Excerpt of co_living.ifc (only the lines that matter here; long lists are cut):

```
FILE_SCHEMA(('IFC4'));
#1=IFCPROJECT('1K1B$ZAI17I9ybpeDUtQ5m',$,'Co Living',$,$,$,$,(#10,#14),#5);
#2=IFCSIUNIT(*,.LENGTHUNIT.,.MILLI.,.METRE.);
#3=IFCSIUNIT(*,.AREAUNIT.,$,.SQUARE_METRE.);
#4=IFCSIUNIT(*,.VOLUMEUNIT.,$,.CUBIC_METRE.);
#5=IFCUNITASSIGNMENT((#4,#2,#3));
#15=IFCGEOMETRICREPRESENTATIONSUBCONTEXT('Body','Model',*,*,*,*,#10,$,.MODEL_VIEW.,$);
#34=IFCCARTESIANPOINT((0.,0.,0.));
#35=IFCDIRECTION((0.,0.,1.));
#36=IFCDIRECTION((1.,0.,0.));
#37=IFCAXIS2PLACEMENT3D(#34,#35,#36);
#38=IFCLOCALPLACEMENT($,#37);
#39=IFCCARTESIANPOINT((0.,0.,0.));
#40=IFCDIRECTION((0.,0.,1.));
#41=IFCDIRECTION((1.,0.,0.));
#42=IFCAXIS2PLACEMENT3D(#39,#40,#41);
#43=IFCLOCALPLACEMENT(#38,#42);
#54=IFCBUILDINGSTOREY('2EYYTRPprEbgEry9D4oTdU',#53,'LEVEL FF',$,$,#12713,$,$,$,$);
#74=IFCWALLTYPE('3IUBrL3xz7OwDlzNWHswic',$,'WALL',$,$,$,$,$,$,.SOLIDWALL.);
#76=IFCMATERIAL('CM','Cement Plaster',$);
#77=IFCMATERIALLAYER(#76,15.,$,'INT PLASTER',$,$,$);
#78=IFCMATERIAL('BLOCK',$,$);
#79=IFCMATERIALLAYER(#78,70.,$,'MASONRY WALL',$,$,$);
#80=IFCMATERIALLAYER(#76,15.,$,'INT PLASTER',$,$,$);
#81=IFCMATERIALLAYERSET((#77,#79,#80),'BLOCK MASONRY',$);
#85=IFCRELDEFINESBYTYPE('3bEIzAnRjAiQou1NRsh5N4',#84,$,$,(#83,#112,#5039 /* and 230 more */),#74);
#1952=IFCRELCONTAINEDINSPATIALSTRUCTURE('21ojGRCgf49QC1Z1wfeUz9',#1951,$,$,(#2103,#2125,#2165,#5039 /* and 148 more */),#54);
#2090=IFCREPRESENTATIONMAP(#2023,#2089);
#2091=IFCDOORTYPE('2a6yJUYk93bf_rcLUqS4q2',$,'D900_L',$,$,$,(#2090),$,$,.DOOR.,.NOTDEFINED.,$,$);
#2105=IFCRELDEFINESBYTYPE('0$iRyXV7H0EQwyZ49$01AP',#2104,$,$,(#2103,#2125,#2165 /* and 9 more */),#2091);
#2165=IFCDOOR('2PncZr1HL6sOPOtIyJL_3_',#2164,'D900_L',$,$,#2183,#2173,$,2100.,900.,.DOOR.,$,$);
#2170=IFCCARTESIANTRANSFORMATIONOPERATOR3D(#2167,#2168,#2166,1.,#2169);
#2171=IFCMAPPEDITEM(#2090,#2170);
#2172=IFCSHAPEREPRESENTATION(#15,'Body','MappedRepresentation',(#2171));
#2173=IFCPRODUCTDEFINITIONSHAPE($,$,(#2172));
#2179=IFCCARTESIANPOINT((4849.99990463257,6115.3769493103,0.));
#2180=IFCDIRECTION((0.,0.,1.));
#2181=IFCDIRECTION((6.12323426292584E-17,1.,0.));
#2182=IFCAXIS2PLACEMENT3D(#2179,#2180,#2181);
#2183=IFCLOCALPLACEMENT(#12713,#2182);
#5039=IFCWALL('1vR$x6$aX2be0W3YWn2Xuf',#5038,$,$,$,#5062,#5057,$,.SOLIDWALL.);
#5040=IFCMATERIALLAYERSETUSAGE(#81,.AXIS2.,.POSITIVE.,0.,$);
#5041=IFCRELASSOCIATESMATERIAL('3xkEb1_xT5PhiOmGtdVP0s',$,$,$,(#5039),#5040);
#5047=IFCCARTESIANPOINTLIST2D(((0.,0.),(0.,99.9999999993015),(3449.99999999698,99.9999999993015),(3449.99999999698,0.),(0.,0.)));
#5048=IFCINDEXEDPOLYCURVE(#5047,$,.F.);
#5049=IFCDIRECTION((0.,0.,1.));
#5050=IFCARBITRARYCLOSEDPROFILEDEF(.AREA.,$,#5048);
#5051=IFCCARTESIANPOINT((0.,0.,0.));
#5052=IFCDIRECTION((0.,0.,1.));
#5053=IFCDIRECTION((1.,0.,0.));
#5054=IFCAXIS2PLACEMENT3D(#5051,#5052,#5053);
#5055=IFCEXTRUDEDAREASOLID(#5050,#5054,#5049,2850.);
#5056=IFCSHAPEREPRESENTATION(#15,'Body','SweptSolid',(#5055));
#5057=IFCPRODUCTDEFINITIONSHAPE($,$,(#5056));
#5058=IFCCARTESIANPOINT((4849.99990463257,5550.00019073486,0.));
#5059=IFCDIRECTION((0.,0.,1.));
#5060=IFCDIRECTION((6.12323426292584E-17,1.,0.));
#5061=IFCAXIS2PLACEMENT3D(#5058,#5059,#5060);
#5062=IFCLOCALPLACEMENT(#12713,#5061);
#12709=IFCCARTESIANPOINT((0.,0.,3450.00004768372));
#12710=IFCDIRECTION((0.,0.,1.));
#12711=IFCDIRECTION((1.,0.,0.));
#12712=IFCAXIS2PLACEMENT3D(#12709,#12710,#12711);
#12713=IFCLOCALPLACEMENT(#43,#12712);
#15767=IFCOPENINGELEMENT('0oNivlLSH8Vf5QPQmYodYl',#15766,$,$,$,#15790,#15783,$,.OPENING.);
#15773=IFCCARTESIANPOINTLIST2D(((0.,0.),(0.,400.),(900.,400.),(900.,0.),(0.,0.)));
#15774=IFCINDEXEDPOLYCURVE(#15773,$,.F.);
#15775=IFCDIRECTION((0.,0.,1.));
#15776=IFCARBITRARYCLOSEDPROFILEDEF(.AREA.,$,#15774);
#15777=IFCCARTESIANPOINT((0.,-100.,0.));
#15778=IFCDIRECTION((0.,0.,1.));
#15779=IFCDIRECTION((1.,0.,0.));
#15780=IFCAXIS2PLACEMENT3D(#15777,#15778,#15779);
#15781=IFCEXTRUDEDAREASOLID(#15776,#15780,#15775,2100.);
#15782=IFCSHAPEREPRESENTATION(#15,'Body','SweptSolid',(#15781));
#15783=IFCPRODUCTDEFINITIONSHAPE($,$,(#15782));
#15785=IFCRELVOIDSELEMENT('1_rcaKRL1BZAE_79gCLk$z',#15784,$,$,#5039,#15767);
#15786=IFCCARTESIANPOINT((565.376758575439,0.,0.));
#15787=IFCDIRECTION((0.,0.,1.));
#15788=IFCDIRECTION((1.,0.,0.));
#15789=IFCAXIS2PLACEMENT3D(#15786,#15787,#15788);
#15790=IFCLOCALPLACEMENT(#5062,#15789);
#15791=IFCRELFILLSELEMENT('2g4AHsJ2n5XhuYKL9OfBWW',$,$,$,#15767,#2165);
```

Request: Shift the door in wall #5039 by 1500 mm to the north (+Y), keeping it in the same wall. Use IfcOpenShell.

```python
import ifcopenshell
import ifcopenshell.api.geometry
import ifcopenshell.util.placement
import ifcopenshell.util.unit

model = ifcopenshell.open("co_living.ifc")
unit_scale = ifcopenshell.util.unit.calculate_unit_scale(model)

door = model.by_guid("2PncZr1HL6sOPOtIyJL_3_")
opening = door.FillsVoids[0].RelatingOpeningElement
wall = opening.VoidsElements[0].RelatingBuildingElement

wall_matrix = ifcopenshell.util.placement.get_local_placement(wall.ObjectPlacement)
shift = wall_matrix[:3, 0] * 1.5 / unit_scale
before = ifcopenshell.util.placement.get_local_placement(door.ObjectPlacement)[:3, 3].copy()

# The door is not placed relative to its opening, so move both.
for product in (opening, door):
    matrix = ifcopenshell.util.placement.get_local_placement(product.ObjectPlacement)
    matrix[:3, 3] += shift
    ifcopenshell.api.geometry.edit_object_placement(model, product=product, matrix=matrix, is_si=False)

after = ifcopenshell.util.placement.get_local_placement(door.ObjectPlacement)[:3, 3]
print("door moved by", (after - before).round(3) + 0.0)

model.write("co_living-out.ifc")
```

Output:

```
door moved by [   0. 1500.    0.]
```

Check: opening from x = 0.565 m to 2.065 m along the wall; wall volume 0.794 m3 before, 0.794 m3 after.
